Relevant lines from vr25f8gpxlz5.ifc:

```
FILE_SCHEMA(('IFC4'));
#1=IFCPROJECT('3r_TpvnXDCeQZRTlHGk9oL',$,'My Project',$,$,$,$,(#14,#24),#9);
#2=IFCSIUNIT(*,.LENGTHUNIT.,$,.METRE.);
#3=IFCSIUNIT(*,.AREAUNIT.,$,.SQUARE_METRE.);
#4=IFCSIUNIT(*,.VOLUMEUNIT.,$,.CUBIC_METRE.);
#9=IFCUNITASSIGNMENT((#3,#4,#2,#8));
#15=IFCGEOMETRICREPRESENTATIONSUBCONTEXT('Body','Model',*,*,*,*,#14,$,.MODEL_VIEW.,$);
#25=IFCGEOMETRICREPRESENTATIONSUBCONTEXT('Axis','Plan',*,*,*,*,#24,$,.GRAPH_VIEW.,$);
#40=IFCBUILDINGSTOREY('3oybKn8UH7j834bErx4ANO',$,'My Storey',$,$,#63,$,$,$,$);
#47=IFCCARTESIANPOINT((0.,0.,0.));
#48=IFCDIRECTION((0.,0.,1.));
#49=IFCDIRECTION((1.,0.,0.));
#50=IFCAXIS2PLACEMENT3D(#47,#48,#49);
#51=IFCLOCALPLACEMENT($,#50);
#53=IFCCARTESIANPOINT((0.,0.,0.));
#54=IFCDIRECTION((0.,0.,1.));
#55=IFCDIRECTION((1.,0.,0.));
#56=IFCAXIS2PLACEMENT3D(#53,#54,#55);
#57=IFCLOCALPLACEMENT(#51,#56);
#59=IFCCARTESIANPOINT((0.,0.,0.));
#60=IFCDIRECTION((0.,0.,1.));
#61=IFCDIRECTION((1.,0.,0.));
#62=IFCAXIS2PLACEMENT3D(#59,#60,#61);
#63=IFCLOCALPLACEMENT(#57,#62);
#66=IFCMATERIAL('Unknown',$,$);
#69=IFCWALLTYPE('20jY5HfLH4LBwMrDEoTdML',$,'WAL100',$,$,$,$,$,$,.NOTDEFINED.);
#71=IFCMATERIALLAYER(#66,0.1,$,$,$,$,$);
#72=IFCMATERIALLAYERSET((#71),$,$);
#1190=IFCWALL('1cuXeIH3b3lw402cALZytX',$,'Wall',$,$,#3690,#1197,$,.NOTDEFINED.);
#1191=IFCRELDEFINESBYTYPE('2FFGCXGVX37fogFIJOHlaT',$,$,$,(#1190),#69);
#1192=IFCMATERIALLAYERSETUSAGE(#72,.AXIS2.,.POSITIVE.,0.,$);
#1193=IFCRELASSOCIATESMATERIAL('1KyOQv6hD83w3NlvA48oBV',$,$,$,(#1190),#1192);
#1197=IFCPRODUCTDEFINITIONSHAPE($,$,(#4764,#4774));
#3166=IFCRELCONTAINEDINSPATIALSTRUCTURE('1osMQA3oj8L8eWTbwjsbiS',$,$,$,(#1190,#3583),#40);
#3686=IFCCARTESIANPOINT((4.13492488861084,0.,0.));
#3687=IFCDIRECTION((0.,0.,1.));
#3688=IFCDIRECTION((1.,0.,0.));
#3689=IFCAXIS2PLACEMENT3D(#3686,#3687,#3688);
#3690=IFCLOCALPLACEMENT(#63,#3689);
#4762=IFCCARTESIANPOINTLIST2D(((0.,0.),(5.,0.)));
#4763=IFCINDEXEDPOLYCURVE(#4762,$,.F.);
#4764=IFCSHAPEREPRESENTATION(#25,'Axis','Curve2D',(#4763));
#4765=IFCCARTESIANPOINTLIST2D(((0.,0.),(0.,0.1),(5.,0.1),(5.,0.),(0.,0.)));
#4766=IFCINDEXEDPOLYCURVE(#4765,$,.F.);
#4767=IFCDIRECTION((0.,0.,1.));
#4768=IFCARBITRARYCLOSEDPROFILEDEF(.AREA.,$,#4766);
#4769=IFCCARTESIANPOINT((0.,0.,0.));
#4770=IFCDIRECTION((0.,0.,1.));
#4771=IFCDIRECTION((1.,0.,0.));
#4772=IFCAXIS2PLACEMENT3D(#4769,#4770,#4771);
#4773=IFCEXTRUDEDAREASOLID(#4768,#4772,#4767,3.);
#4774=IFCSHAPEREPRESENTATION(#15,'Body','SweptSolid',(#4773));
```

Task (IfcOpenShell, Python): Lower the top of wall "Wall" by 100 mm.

```python
import ifcopenshell
import ifcopenshell.geom
import ifcopenshell.util.representation
import ifcopenshell.util.shape
import ifcopenshell.util.unit

model = ifcopenshell.open("vr25f8gpxlz5.ifc")
unit_scale = ifcopenshell.util.unit.calculate_unit_scale(model)
settings = ifcopenshell.geom.settings()


def volume(element):
    """Net volume in cubic metres, openings subtracted."""
    shape = ifcopenshell.geom.create_shape(settings, element)
    return ifcopenshell.util.shape.get_volume(shape.geometry)


wall = model.by_guid("1cuXeIH3b3lw402cALZytX")
before = volume(wall)

body = ifcopenshell.util.representation.get_representation(wall, "Model", "Body")
solid = body.Items[0]
old_height = solid.Depth
solid.Depth -= 0.1 / unit_scale
after = volume(wall)

print(f"height {old_height:g} -> {solid.Depth:g}, volume {before:.3f} -> {after:.3f} m3")

model.write("vr25f8gpxlz5_rev.ifc")
```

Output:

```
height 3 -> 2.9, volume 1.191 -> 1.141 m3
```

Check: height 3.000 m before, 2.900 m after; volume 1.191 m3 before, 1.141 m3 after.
